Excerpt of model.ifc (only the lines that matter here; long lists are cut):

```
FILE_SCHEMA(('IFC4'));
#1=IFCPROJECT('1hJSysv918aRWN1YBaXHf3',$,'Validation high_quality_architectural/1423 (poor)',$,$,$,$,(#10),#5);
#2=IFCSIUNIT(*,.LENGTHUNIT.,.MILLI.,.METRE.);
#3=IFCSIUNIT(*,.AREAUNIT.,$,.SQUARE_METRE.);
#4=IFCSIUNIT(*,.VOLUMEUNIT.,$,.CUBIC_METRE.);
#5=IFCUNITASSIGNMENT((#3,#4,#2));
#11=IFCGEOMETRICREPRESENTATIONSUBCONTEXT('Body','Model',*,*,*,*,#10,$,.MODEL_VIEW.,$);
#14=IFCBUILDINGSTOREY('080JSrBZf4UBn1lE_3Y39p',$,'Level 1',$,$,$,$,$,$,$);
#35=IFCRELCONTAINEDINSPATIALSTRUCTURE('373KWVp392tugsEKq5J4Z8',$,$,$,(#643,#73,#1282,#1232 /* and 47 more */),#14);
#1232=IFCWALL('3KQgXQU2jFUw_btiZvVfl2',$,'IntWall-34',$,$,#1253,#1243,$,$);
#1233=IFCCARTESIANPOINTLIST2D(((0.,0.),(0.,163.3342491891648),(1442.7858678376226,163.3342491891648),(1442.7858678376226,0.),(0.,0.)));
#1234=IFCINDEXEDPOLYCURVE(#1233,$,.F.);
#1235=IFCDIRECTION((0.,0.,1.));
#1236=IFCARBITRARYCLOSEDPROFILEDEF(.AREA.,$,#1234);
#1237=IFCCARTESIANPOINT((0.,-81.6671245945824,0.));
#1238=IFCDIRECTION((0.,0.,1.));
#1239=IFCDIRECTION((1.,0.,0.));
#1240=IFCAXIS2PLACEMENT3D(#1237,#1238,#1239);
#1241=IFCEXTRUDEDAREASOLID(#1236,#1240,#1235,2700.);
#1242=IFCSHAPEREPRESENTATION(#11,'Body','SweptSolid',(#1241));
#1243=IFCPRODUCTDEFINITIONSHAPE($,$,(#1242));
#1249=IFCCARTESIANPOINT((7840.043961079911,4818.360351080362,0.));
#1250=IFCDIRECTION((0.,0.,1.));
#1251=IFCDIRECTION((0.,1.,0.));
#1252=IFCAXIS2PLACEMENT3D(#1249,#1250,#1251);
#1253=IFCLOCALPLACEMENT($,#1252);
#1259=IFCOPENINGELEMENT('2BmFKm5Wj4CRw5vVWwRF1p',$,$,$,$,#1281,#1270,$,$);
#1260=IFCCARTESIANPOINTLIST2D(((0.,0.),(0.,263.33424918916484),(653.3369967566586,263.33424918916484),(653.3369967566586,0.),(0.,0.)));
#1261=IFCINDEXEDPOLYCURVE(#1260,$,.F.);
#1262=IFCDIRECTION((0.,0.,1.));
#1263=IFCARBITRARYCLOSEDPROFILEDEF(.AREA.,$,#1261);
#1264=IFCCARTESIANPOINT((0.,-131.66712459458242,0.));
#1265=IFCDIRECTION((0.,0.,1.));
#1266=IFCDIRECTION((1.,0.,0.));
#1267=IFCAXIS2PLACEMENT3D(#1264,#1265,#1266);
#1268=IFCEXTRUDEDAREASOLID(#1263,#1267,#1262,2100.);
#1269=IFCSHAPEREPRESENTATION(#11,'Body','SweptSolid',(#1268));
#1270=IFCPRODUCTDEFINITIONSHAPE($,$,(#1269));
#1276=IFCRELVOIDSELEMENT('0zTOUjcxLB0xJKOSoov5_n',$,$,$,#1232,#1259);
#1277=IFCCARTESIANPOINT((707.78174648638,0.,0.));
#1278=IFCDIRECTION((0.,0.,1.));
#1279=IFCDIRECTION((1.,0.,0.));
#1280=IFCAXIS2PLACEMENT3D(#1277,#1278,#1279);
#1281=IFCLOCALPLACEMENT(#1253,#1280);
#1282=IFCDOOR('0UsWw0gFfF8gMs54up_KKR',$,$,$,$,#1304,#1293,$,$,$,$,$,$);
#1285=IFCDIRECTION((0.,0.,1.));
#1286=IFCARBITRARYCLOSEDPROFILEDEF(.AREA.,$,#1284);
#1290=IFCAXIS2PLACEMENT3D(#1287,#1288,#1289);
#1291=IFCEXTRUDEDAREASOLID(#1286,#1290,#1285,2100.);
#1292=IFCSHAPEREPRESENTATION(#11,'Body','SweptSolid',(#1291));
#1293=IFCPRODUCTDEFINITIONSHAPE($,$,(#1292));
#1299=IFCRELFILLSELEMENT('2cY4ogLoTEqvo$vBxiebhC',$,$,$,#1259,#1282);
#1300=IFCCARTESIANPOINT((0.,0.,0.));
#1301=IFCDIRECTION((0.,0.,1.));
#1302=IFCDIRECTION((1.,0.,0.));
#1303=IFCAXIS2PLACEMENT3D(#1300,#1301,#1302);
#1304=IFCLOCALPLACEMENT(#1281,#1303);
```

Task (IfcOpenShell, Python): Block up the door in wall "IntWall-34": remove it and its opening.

```python
import ifcopenshell
import ifcopenshell.api.feature
import ifcopenshell.api.root
import ifcopenshell.geom
import ifcopenshell.util.shape

model = ifcopenshell.open("model.ifc")
settings = ifcopenshell.geom.settings()


def volume(element):
    """Net volume in cubic metres, openings subtracted."""
    shape = ifcopenshell.geom.create_shape(settings, element)
    return ifcopenshell.util.shape.get_volume(shape.geometry)


door = model.by_guid("0UsWw0gFfF8gMs54up_KKR")
opening = door.FillsVoids[0].RelatingOpeningElement
wall = opening.VoidsElements[0].RelatingBuildingElement
before = volume(wall)

ifcopenshell.api.root.remove_product(model, product=door)
ifcopenshell.api.feature.remove_feature(model, feature=opening)

after = volume(wall)

print(f"wall volume {before:.3f} -> {after:.3f} m3")

model.write("model_rev.ifc")
```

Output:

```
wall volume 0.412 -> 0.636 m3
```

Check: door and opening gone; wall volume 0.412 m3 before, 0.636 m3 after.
